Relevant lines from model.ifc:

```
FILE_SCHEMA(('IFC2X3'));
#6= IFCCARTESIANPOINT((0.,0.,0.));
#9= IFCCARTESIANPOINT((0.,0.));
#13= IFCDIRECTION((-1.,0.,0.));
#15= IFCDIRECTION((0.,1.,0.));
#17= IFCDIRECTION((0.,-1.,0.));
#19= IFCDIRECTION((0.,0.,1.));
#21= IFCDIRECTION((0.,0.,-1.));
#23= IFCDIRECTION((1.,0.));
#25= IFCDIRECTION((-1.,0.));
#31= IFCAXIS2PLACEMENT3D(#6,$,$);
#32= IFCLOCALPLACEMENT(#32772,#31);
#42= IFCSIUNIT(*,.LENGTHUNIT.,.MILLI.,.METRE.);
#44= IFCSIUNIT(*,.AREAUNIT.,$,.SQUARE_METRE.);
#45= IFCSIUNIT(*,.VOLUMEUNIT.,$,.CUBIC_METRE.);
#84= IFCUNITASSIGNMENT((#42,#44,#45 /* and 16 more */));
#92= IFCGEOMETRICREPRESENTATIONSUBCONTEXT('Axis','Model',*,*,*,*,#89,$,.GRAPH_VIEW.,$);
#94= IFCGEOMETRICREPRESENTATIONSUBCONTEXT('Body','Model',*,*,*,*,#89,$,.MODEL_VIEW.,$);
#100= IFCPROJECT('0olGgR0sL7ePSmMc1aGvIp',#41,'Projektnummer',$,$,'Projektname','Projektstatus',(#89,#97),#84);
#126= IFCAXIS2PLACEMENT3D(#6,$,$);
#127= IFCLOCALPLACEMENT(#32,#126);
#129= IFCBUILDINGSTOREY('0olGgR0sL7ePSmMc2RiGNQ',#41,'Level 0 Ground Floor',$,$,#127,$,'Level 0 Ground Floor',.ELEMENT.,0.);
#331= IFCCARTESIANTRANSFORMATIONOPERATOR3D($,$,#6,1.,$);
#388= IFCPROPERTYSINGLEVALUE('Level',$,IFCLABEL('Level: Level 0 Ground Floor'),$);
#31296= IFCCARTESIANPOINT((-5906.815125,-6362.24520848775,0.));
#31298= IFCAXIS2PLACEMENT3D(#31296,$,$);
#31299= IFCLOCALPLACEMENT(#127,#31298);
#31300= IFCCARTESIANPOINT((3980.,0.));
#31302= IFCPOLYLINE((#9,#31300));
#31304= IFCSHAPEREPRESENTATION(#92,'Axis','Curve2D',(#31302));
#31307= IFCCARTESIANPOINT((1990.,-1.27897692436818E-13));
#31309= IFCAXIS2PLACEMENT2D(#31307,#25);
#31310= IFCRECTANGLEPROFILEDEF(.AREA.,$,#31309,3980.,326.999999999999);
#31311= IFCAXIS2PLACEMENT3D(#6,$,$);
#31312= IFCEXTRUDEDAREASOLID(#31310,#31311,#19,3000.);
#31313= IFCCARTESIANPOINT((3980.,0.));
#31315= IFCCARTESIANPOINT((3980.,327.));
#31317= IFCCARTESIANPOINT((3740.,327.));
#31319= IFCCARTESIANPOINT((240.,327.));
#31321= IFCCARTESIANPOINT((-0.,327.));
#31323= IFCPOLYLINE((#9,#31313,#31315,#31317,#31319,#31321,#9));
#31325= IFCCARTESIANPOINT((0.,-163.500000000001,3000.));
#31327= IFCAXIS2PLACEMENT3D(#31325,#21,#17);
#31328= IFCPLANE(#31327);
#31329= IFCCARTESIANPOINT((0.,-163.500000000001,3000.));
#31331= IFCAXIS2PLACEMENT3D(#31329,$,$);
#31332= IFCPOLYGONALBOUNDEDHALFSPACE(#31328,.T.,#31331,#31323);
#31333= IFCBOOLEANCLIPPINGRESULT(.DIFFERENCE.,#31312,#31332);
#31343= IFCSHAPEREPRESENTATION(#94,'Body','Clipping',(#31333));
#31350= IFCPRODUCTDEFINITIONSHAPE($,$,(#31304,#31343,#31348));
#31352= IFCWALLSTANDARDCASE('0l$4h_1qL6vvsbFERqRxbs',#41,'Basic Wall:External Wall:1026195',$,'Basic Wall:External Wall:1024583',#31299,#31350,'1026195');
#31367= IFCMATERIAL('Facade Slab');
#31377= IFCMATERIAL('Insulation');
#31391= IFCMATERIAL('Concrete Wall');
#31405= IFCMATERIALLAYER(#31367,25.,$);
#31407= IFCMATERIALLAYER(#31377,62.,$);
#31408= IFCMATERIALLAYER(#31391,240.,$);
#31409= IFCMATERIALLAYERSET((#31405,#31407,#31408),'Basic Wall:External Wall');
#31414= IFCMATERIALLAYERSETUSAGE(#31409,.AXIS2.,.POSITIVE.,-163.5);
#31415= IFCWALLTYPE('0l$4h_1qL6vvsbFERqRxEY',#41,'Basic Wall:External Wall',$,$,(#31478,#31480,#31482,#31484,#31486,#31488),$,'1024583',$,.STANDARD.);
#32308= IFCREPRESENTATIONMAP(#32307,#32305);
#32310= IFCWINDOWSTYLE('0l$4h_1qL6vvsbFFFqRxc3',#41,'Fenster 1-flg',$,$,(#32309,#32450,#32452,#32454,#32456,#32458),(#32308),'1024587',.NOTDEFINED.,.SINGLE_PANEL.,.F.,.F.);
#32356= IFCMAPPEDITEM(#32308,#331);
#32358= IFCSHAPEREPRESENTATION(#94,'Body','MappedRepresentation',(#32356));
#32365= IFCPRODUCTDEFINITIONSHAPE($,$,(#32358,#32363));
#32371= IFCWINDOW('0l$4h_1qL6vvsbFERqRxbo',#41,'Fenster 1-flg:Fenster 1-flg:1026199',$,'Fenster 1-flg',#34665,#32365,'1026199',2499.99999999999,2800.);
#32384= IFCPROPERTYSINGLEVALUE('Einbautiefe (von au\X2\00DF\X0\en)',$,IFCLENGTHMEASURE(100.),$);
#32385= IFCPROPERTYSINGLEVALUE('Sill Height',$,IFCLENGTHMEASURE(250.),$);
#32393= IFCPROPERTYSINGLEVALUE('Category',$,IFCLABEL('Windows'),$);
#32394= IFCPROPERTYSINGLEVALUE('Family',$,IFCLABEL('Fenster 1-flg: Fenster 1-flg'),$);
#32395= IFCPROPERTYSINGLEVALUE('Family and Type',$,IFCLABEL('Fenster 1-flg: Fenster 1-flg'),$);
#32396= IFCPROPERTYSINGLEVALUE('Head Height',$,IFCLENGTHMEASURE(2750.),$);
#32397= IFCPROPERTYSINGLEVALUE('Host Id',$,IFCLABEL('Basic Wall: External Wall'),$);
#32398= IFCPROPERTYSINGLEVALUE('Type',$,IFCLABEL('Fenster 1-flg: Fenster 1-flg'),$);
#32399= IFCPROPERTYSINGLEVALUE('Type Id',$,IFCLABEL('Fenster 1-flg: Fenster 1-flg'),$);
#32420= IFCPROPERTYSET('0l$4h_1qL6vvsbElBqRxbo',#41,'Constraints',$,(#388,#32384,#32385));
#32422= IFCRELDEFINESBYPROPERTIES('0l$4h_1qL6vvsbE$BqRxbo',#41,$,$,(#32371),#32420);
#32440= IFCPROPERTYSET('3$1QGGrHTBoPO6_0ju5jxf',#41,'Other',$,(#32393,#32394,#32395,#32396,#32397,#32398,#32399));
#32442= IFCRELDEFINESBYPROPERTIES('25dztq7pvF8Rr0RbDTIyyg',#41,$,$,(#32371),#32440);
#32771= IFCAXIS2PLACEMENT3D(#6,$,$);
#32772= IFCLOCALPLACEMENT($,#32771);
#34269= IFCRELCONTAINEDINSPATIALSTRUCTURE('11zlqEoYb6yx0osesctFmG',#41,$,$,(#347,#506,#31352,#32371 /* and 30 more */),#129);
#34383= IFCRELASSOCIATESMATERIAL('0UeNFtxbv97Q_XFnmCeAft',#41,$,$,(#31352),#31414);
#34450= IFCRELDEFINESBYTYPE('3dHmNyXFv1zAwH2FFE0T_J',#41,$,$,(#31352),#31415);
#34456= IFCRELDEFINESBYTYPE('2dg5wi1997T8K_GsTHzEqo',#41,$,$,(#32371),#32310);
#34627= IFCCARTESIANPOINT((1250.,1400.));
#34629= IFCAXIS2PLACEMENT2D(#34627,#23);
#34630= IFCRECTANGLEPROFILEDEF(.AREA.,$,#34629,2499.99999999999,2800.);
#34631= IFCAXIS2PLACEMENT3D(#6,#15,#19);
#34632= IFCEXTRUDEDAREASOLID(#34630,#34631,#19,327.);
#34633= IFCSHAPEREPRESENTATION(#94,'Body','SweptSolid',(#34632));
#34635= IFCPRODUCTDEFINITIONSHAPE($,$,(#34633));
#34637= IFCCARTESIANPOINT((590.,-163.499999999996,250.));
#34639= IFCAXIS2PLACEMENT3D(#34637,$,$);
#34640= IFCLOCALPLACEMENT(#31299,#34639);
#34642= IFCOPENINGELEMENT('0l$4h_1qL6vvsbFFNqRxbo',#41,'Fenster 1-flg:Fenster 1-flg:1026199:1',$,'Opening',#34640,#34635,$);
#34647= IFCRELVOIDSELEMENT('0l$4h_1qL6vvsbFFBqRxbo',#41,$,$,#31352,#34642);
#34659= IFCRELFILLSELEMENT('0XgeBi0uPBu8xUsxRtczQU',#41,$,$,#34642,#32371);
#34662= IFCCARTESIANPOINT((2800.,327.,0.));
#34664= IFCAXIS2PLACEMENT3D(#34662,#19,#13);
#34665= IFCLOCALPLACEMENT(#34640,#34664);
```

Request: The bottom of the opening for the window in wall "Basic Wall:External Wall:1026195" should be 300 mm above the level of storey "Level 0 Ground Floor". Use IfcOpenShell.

```python
import numpy as np
import ifcopenshell
import ifcopenshell.api.geometry
import ifcopenshell.api.pset
import ifcopenshell.geom
import ifcopenshell.util.element
import ifcopenshell.util.placement
import ifcopenshell.util.shape
import ifcopenshell.util.unit

model = ifcopenshell.open("model.ifc")
unit_scale = ifcopenshell.util.unit.calculate_unit_scale(model)

window = model.by_guid("0l$4h_1qL6vvsbFERqRxbo")
opening = window.FillsVoids[0].RelatingOpeningElement
storey = ifcopenshell.util.element.get_container(window, ifc_class="IfcBuildingStorey")
level = ifcopenshell.util.placement.get_local_placement(storey.ObjectPlacement)[2, 3]

# The opening's origin need not be at the sill, so measure its lowest point.
shape = ifcopenshell.geom.create_shape(ifcopenshell.geom.settings(), opening)
bottom = ifcopenshell.util.shape.get_shape_bottom_elevation(shape, shape.geometry) / unit_scale
dz = level + 300.0 - bottom

shift = np.array([0.0, 0.0, dz])
# The window is placed relative to its opening, so it follows when the opening moves.
matrix = ifcopenshell.util.placement.get_local_placement(opening.ObjectPlacement)
matrix[:3, 3] += shift
ifcopenshell.api.geometry.edit_object_placement(
    model, product=opening, matrix=matrix, is_si=False, should_transform_children=True
)

# Keep the stored heights in step.
pset = model.by_id(ifcopenshell.util.element.get_pset(window, "Constraints", should_inherit=False)["id"])
ifcopenshell.api.pset.edit_pset(model, pset=pset, properties={
    "Sill Height": model.create_entity("IfcLengthMeasure", ifcopenshell.util.element.get_pset(window, "Constraints", "Sill Height") + dz),
})
pset = model.by_id(ifcopenshell.util.element.get_pset(window, "Other", should_inherit=False)["id"])
ifcopenshell.api.pset.edit_pset(model, pset=pset, properties={
    "Head Height": model.create_entity("IfcLengthMeasure", ifcopenshell.util.element.get_pset(window, "Other", "Head Height") + dz),
})

print(f"moved by {dz * unit_scale:+.3f} m")

model.write("model_updated.ifc")
```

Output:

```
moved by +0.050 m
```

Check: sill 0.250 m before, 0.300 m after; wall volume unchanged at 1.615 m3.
